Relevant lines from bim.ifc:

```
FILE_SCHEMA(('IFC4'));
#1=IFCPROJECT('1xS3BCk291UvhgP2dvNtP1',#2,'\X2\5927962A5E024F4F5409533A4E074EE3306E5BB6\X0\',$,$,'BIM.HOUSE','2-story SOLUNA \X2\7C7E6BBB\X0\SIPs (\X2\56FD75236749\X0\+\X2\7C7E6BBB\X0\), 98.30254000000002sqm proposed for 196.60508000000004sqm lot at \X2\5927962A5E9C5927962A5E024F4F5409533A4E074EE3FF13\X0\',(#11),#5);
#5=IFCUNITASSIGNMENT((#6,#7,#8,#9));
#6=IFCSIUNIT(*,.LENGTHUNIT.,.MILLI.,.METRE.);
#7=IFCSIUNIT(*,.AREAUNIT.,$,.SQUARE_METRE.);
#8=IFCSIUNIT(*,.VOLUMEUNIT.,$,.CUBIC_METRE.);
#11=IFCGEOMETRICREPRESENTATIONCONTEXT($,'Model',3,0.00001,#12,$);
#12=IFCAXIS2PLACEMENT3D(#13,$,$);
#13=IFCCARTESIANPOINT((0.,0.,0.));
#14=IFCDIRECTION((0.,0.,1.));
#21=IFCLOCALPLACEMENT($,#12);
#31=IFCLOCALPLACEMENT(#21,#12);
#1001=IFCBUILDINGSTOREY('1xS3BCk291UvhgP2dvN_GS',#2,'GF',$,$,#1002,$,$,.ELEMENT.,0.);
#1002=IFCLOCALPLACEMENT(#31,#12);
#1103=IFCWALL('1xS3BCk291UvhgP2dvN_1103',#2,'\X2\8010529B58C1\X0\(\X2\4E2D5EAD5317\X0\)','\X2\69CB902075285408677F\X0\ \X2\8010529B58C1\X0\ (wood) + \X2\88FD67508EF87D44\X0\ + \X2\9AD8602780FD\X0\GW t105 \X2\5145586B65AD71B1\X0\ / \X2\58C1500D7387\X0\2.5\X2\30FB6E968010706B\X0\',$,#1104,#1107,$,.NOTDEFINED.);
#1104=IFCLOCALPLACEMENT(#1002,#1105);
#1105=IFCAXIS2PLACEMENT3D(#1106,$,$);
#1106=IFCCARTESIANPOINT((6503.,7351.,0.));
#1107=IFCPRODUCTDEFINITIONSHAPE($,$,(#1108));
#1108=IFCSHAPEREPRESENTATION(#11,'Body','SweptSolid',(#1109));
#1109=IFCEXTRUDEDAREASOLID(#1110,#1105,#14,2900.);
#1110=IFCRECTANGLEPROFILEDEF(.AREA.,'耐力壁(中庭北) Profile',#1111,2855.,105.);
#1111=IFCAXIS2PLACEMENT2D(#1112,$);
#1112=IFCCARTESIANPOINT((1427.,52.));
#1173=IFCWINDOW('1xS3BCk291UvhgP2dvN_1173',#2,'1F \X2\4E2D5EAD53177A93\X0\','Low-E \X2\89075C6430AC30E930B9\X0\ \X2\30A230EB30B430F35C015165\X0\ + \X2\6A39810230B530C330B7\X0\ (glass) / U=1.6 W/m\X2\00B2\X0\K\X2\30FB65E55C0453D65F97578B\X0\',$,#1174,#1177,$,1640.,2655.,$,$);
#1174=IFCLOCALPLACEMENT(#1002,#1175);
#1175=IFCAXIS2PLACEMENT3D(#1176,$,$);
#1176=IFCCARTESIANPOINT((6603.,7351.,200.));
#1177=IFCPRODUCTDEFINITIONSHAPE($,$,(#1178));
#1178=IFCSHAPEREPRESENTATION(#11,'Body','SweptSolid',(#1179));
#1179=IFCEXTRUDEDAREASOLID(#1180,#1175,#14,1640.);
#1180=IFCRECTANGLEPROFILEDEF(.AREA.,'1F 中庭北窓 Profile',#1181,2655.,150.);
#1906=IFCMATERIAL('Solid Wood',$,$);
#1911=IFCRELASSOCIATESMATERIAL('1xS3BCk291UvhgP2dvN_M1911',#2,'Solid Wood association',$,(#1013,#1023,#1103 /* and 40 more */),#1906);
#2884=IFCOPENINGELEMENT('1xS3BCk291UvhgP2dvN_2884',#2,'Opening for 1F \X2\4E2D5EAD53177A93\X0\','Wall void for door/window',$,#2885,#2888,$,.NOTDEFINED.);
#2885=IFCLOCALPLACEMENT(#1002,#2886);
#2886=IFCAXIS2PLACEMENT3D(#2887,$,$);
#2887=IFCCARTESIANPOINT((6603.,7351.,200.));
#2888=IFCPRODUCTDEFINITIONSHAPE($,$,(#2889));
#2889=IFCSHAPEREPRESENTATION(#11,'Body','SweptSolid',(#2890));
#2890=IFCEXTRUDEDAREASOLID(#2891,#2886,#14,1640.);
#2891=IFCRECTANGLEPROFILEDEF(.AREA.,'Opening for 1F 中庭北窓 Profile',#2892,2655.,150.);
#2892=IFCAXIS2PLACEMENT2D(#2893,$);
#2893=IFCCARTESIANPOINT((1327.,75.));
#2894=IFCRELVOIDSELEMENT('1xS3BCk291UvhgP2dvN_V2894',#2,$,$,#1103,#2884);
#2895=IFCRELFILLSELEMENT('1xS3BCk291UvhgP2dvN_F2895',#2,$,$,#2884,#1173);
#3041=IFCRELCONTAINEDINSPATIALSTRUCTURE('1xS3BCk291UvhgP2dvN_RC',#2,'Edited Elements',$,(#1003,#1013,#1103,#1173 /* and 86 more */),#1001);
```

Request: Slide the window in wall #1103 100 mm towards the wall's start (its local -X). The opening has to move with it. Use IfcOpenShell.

```python
import ifcopenshell
import ifcopenshell.api.geometry
import ifcopenshell.util.placement
import ifcopenshell.util.unit

model = ifcopenshell.open("bim.ifc")
unit_scale = ifcopenshell.util.unit.calculate_unit_scale(model)

window = model.by_guid("1xS3BCk291UvhgP2dvN_1173")
opening = window.FillsVoids[0].RelatingOpeningElement
wall = opening.VoidsElements[0].RelatingBuildingElement

wall_matrix = ifcopenshell.util.placement.get_local_placement(wall.ObjectPlacement)
shift = wall_matrix[:3, 0] * -0.1 / unit_scale
before = ifcopenshell.util.placement.get_local_placement(window.ObjectPlacement)[:3, 3].copy()

# The window is not placed relative to its opening, so move both.
for product in (opening, window):
    matrix = ifcopenshell.util.placement.get_local_placement(product.ObjectPlacement)
    matrix[:3, 3] += shift
    ifcopenshell.api.geometry.edit_object_placement(model, product=product, matrix=matrix, is_si=False)

after = ifcopenshell.util.placement.get_local_placement(window.ObjectPlacement)[:3, 3]
print("window moved by", (after - before).round(3) + 0.0)

model.write("bim_v2.ifc")
```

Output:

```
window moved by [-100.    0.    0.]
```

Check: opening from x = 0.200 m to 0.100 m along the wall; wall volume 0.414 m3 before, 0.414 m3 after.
